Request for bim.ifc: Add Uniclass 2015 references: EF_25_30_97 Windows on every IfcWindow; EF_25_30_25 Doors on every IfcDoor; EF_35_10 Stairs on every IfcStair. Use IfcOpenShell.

First a look at what the model holds.

```python
import ifcopenshell

model = ifcopenshell.open("bim.ifc")
print(model.schema)
print("classifications:", [c.Name for c in model.by_type("IfcClassification")])
for ifc_class in ("IfcDoor", "IfcRoof", "IfcStair", "IfcWall", "IfcWindow"):
    print(ifc_class, len(model.by_type(ifc_class)))
```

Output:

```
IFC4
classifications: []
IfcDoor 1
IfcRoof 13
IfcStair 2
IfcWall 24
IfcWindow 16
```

```python
import ifcopenshell
import ifcopenshell.api.classification

model = ifcopenshell.open("bim.ifc")

system = ifcopenshell.api.classification.add_classification(model, classification="Uniclass 2015")

codes = {
    "IfcWindow": ("EF_25_30_97", "Windows"),
    "IfcDoor": ("EF_25_30_25", "Doors"),
    "IfcStair": ("EF_35_10", "Stairs"),
}
for ifc_class, (code, name) in codes.items():
    products = model.by_type(ifc_class)
    ifcopenshell.api.classification.add_reference(
        model, products=products, classification=system, identification=code, name=name
    )
    print(code, len(products))

model.write("bim_updated.ifc")
```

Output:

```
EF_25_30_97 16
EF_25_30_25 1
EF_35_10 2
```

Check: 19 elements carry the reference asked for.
